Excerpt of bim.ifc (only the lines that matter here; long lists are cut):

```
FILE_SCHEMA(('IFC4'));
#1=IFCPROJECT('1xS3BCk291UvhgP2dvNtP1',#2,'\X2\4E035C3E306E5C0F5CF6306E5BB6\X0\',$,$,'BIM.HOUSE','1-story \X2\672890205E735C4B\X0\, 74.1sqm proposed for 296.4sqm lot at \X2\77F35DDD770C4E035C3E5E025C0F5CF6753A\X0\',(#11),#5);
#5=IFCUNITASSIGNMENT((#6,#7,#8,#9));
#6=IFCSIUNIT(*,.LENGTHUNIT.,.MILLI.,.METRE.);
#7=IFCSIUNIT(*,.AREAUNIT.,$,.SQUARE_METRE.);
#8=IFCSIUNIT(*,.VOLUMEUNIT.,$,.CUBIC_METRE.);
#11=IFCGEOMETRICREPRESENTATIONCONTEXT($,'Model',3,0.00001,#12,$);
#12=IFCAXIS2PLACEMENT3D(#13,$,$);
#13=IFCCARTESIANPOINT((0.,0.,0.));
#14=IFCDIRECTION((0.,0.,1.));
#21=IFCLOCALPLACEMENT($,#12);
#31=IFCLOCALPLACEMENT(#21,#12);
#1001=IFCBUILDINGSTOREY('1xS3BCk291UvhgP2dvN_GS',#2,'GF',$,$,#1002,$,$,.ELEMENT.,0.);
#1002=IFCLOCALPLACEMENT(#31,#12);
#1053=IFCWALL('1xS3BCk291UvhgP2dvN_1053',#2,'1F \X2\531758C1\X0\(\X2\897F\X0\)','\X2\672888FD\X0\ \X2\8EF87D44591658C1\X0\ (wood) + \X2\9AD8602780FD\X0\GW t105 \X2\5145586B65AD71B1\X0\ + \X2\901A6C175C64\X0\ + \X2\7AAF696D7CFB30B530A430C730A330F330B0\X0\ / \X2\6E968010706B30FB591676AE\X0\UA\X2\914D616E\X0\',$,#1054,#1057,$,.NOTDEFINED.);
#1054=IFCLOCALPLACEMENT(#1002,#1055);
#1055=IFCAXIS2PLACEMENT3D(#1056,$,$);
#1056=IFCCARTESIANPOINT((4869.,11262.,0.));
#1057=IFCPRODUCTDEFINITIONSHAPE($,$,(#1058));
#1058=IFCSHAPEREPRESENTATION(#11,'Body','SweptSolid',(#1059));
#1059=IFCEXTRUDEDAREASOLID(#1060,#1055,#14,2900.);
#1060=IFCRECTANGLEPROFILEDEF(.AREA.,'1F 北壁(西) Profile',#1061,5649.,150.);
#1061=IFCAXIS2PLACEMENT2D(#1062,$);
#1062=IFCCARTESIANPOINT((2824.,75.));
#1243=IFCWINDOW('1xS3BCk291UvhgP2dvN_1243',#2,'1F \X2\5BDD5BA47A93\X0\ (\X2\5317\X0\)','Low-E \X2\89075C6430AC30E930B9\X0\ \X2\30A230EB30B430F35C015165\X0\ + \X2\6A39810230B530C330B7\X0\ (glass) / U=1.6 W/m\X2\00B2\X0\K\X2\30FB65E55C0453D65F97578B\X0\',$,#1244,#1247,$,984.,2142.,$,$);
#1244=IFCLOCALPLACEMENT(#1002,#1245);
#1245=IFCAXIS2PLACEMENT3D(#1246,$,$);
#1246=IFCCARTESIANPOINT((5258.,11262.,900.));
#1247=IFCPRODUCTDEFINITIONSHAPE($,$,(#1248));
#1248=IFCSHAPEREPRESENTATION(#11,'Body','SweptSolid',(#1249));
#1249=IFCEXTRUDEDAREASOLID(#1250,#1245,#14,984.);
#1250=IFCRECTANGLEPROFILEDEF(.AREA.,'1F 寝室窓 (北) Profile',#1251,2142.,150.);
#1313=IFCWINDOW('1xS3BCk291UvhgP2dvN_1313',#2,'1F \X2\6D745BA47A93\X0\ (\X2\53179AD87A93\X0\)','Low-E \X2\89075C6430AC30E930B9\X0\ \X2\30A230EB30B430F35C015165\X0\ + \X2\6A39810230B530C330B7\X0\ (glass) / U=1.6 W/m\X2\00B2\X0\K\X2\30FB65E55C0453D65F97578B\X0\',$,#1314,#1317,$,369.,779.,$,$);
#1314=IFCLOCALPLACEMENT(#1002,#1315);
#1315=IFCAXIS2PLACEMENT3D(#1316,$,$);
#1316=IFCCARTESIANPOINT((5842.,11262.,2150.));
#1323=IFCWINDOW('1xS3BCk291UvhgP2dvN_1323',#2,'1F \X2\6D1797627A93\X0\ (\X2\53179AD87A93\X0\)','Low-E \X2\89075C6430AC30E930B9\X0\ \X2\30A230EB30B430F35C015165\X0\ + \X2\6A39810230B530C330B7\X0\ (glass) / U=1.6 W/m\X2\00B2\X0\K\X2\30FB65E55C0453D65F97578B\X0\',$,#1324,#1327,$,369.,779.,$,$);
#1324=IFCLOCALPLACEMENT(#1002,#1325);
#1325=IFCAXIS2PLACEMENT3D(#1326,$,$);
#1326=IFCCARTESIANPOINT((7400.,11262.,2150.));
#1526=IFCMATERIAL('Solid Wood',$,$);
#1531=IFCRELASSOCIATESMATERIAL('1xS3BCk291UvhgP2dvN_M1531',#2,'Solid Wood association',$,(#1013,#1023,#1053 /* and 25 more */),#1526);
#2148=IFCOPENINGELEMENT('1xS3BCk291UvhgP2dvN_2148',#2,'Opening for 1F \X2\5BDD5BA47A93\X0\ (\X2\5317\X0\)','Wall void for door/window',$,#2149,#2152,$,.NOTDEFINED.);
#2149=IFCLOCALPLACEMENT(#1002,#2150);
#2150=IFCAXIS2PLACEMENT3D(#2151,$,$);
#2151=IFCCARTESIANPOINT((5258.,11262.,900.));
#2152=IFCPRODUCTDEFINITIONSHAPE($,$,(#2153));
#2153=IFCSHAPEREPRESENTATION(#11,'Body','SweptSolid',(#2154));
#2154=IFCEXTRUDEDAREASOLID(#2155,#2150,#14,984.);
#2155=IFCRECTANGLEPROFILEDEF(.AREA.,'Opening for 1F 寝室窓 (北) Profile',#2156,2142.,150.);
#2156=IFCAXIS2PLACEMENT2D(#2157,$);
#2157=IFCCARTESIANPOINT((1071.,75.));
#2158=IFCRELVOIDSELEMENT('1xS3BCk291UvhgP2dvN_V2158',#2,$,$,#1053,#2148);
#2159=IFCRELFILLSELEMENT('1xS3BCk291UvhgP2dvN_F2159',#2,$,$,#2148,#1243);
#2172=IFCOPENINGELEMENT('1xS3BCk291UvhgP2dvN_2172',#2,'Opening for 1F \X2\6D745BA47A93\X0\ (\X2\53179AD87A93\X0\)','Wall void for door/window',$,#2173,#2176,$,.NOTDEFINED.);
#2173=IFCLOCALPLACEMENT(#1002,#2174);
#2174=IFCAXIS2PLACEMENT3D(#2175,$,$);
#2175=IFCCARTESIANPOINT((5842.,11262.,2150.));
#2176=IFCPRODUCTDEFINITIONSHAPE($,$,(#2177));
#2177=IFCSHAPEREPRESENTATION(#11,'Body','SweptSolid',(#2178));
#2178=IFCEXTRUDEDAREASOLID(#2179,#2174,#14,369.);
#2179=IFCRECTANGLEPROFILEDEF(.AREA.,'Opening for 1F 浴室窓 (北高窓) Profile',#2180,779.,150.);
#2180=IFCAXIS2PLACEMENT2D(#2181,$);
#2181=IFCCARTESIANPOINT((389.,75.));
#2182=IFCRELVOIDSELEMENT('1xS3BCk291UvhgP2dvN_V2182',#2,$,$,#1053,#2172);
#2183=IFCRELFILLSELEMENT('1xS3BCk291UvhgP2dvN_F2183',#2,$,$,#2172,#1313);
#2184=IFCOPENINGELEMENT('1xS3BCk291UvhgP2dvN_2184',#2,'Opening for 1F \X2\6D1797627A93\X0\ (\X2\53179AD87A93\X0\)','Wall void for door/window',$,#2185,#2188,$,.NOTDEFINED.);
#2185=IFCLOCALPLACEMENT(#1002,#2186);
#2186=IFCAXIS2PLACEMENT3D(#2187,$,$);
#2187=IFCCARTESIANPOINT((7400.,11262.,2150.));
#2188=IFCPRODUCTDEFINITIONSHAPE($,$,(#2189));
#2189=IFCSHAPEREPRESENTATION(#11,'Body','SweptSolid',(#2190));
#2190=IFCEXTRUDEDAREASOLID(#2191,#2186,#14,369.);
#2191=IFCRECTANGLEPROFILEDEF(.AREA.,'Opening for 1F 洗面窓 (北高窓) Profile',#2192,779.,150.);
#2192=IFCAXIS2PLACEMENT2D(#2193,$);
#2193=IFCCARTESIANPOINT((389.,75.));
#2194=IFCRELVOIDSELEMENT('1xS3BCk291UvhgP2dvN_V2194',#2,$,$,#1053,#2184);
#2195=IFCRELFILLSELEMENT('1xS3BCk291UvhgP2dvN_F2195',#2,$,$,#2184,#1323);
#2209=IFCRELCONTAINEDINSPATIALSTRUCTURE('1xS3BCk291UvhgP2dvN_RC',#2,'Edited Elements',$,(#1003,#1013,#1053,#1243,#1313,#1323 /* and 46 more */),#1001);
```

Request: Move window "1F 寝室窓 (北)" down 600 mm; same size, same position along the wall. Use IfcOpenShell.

```python
import numpy as np
import ifcopenshell
import ifcopenshell.api.geometry
import ifcopenshell.util.placement
import ifcopenshell.util.unit

model = ifcopenshell.open("bim.ifc")
unit_scale = ifcopenshell.util.unit.calculate_unit_scale(model)

window = model.by_guid("1xS3BCk291UvhgP2dvN_1243")
opening = window.FillsVoids[0].RelatingOpeningElement
dz = -0.6 / unit_scale

shift = np.array([0.0, 0.0, dz])
# The window is not placed relative to its opening, so move both.
for product in (opening, window):
    matrix = ifcopenshell.util.placement.get_local_placement(product.ObjectPlacement)
    matrix[:3, 3] += shift
    ifcopenshell.api.geometry.edit_object_placement(model, product=product, matrix=matrix, is_si=False)

print(f"moved by {dz * unit_scale:+.3f} m")

model.write("bim_updated.ifc")
```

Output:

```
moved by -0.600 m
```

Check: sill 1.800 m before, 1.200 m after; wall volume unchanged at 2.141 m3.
